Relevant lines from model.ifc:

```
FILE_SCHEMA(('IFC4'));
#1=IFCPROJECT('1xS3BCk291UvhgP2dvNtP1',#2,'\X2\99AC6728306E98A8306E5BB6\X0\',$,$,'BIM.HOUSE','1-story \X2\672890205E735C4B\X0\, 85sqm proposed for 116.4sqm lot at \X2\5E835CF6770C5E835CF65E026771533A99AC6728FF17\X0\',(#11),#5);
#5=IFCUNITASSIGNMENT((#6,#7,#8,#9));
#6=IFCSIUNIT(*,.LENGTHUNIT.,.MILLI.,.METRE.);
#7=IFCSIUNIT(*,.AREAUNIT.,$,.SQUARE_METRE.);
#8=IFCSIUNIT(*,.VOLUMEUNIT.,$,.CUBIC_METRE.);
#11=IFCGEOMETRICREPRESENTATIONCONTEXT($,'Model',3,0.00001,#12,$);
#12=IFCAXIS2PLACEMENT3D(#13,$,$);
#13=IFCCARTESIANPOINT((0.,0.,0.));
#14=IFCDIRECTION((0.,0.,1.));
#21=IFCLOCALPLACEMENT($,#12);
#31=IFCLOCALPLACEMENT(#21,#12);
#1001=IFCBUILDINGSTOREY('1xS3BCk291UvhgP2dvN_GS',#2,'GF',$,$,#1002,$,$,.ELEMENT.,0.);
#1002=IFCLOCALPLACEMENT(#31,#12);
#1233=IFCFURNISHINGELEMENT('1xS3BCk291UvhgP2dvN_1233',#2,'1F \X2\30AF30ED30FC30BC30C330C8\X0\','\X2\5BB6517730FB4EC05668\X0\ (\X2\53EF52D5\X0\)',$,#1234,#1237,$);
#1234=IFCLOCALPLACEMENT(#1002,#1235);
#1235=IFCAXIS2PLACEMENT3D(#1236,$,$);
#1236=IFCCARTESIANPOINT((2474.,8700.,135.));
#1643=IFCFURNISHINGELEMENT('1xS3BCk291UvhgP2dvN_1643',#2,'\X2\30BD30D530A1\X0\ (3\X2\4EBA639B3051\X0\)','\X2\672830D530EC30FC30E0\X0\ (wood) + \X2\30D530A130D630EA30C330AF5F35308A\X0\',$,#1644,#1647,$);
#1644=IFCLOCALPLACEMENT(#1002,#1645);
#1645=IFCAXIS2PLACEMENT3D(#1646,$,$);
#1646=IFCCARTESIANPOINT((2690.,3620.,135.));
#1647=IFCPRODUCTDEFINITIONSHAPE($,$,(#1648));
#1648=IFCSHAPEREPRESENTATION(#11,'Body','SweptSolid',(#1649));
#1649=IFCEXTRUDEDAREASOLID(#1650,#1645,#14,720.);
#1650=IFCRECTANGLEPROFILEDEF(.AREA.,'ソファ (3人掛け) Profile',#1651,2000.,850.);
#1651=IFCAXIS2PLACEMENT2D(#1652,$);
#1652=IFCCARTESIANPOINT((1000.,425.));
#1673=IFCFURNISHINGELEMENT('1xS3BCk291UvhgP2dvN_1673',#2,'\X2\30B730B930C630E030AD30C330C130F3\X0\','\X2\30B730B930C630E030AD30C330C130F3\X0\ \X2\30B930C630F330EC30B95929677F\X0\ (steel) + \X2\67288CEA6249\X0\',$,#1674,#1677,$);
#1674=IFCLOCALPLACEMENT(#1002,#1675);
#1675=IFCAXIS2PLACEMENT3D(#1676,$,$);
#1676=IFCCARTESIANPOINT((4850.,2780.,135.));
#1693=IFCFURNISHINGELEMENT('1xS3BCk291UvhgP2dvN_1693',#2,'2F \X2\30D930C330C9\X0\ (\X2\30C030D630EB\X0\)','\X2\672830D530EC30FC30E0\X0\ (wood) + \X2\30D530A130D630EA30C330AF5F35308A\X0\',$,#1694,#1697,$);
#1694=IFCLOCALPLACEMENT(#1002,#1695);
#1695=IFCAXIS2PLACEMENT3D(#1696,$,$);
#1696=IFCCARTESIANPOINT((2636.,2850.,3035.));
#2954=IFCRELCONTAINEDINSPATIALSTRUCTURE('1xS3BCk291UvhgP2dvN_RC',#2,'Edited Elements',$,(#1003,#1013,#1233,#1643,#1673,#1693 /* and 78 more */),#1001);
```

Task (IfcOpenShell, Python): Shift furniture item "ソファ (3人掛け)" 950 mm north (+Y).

```python
import ifcopenshell
import ifcopenshell.api.geometry
import ifcopenshell.util.placement
import ifcopenshell.util.unit

model = ifcopenshell.open("model.ifc")
unit_scale = ifcopenshell.util.unit.calculate_unit_scale(model)

item = model.by_id(1643)
matrix = ifcopenshell.util.placement.get_local_placement(item.ObjectPlacement)
matrix[1, 3] += 0.95 / unit_scale
ifcopenshell.api.geometry.edit_object_placement(model, product=item, matrix=matrix, is_si=False)

print(ifcopenshell.util.placement.get_local_placement(item.ObjectPlacement).round(3) + 0.0)

model.write("model_edited.ifc")
```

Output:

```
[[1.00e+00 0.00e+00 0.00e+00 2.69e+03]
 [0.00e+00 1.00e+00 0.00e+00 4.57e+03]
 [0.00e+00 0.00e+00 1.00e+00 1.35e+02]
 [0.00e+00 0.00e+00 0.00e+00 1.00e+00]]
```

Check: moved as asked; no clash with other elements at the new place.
